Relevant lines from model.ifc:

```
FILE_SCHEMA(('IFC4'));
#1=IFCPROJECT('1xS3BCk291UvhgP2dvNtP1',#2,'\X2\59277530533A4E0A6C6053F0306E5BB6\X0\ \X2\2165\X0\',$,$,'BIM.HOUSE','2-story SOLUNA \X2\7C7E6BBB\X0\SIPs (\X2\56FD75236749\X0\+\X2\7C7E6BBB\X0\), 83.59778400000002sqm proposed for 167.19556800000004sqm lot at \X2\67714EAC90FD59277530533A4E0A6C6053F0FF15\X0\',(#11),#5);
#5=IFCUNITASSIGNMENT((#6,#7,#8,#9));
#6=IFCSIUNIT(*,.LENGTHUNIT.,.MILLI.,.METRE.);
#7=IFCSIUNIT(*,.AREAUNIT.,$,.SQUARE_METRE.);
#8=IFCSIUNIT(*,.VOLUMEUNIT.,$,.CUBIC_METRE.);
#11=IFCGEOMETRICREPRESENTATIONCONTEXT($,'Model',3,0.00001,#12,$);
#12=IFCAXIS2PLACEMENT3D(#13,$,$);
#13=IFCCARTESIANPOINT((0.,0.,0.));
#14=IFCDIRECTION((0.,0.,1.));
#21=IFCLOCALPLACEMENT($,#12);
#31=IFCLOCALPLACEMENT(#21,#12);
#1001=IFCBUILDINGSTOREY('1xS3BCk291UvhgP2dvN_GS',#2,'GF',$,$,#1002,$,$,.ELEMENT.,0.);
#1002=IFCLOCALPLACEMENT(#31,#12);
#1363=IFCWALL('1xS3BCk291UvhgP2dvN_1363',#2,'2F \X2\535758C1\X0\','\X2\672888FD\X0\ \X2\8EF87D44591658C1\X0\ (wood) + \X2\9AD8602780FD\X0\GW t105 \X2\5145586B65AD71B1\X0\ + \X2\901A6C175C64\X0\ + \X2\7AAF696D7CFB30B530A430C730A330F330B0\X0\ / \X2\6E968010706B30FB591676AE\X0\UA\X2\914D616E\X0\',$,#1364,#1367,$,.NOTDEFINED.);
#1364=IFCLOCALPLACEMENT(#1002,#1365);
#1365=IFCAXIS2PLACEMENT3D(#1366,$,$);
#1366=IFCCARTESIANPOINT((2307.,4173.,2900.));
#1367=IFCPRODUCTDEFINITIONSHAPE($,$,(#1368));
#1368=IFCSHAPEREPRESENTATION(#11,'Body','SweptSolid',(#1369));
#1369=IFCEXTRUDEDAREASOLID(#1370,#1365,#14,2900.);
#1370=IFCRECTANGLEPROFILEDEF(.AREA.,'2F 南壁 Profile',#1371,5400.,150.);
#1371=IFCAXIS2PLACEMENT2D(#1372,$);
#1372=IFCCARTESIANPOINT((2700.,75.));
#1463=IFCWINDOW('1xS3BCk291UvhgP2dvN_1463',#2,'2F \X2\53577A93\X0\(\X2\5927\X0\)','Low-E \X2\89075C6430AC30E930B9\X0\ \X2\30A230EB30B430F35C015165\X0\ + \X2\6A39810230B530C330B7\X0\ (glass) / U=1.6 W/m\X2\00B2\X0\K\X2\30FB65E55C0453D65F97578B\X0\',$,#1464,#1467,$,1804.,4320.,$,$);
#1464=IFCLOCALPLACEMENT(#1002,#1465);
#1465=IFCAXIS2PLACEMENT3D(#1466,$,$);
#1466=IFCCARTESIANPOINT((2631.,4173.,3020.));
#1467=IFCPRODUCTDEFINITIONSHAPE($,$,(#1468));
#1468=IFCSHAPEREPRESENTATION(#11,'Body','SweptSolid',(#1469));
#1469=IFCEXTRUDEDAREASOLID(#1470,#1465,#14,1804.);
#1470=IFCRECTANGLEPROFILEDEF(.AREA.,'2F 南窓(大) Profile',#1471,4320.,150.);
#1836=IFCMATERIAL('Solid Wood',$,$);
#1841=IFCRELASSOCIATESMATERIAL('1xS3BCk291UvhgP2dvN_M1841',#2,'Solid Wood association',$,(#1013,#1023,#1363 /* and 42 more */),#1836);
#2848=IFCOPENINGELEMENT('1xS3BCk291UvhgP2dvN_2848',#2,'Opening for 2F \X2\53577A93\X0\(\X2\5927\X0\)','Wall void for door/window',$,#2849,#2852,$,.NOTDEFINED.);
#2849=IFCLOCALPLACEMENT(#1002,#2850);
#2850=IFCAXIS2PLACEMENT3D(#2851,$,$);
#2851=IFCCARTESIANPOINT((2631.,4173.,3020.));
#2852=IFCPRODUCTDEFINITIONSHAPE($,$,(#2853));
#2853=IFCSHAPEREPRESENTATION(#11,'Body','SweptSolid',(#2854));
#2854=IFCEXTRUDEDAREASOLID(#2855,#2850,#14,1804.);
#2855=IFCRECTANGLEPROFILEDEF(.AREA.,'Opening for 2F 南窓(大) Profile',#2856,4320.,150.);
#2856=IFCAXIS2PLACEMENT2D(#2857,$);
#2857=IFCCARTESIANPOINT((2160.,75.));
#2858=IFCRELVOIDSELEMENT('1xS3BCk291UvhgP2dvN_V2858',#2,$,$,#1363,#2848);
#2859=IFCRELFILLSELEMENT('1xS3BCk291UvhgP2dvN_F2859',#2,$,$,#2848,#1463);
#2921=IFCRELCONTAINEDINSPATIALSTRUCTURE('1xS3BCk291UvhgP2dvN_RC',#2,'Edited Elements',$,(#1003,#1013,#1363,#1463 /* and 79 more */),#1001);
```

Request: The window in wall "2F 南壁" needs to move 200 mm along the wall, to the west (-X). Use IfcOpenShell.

```python
import ifcopenshell
import ifcopenshell.api.geometry
import ifcopenshell.util.placement
import ifcopenshell.util.unit

model = ifcopenshell.open("model.ifc")
unit_scale = ifcopenshell.util.unit.calculate_unit_scale(model)

window = model.by_guid("1xS3BCk291UvhgP2dvN_1463")
opening = window.FillsVoids[0].RelatingOpeningElement
wall = opening.VoidsElements[0].RelatingBuildingElement

wall_matrix = ifcopenshell.util.placement.get_local_placement(wall.ObjectPlacement)
shift = wall_matrix[:3, 0] * -0.2 / unit_scale
before = ifcopenshell.util.placement.get_local_placement(window.ObjectPlacement)[:3, 3].copy()

# The window is not placed relative to its opening, so move both.
for product in (opening, window):
    matrix = ifcopenshell.util.placement.get_local_placement(product.ObjectPlacement)
    matrix[:3, 3] += shift
    ifcopenshell.api.geometry.edit_object_placement(model, product=product, matrix=matrix, is_si=False)

after = ifcopenshell.util.placement.get_local_placement(window.ObjectPlacement)[:3, 3]
print("window moved by", (after - before).round(3) + 0.0)

model.write("model_v2.ifc")
```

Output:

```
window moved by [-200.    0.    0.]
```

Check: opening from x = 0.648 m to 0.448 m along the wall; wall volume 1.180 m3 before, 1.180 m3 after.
